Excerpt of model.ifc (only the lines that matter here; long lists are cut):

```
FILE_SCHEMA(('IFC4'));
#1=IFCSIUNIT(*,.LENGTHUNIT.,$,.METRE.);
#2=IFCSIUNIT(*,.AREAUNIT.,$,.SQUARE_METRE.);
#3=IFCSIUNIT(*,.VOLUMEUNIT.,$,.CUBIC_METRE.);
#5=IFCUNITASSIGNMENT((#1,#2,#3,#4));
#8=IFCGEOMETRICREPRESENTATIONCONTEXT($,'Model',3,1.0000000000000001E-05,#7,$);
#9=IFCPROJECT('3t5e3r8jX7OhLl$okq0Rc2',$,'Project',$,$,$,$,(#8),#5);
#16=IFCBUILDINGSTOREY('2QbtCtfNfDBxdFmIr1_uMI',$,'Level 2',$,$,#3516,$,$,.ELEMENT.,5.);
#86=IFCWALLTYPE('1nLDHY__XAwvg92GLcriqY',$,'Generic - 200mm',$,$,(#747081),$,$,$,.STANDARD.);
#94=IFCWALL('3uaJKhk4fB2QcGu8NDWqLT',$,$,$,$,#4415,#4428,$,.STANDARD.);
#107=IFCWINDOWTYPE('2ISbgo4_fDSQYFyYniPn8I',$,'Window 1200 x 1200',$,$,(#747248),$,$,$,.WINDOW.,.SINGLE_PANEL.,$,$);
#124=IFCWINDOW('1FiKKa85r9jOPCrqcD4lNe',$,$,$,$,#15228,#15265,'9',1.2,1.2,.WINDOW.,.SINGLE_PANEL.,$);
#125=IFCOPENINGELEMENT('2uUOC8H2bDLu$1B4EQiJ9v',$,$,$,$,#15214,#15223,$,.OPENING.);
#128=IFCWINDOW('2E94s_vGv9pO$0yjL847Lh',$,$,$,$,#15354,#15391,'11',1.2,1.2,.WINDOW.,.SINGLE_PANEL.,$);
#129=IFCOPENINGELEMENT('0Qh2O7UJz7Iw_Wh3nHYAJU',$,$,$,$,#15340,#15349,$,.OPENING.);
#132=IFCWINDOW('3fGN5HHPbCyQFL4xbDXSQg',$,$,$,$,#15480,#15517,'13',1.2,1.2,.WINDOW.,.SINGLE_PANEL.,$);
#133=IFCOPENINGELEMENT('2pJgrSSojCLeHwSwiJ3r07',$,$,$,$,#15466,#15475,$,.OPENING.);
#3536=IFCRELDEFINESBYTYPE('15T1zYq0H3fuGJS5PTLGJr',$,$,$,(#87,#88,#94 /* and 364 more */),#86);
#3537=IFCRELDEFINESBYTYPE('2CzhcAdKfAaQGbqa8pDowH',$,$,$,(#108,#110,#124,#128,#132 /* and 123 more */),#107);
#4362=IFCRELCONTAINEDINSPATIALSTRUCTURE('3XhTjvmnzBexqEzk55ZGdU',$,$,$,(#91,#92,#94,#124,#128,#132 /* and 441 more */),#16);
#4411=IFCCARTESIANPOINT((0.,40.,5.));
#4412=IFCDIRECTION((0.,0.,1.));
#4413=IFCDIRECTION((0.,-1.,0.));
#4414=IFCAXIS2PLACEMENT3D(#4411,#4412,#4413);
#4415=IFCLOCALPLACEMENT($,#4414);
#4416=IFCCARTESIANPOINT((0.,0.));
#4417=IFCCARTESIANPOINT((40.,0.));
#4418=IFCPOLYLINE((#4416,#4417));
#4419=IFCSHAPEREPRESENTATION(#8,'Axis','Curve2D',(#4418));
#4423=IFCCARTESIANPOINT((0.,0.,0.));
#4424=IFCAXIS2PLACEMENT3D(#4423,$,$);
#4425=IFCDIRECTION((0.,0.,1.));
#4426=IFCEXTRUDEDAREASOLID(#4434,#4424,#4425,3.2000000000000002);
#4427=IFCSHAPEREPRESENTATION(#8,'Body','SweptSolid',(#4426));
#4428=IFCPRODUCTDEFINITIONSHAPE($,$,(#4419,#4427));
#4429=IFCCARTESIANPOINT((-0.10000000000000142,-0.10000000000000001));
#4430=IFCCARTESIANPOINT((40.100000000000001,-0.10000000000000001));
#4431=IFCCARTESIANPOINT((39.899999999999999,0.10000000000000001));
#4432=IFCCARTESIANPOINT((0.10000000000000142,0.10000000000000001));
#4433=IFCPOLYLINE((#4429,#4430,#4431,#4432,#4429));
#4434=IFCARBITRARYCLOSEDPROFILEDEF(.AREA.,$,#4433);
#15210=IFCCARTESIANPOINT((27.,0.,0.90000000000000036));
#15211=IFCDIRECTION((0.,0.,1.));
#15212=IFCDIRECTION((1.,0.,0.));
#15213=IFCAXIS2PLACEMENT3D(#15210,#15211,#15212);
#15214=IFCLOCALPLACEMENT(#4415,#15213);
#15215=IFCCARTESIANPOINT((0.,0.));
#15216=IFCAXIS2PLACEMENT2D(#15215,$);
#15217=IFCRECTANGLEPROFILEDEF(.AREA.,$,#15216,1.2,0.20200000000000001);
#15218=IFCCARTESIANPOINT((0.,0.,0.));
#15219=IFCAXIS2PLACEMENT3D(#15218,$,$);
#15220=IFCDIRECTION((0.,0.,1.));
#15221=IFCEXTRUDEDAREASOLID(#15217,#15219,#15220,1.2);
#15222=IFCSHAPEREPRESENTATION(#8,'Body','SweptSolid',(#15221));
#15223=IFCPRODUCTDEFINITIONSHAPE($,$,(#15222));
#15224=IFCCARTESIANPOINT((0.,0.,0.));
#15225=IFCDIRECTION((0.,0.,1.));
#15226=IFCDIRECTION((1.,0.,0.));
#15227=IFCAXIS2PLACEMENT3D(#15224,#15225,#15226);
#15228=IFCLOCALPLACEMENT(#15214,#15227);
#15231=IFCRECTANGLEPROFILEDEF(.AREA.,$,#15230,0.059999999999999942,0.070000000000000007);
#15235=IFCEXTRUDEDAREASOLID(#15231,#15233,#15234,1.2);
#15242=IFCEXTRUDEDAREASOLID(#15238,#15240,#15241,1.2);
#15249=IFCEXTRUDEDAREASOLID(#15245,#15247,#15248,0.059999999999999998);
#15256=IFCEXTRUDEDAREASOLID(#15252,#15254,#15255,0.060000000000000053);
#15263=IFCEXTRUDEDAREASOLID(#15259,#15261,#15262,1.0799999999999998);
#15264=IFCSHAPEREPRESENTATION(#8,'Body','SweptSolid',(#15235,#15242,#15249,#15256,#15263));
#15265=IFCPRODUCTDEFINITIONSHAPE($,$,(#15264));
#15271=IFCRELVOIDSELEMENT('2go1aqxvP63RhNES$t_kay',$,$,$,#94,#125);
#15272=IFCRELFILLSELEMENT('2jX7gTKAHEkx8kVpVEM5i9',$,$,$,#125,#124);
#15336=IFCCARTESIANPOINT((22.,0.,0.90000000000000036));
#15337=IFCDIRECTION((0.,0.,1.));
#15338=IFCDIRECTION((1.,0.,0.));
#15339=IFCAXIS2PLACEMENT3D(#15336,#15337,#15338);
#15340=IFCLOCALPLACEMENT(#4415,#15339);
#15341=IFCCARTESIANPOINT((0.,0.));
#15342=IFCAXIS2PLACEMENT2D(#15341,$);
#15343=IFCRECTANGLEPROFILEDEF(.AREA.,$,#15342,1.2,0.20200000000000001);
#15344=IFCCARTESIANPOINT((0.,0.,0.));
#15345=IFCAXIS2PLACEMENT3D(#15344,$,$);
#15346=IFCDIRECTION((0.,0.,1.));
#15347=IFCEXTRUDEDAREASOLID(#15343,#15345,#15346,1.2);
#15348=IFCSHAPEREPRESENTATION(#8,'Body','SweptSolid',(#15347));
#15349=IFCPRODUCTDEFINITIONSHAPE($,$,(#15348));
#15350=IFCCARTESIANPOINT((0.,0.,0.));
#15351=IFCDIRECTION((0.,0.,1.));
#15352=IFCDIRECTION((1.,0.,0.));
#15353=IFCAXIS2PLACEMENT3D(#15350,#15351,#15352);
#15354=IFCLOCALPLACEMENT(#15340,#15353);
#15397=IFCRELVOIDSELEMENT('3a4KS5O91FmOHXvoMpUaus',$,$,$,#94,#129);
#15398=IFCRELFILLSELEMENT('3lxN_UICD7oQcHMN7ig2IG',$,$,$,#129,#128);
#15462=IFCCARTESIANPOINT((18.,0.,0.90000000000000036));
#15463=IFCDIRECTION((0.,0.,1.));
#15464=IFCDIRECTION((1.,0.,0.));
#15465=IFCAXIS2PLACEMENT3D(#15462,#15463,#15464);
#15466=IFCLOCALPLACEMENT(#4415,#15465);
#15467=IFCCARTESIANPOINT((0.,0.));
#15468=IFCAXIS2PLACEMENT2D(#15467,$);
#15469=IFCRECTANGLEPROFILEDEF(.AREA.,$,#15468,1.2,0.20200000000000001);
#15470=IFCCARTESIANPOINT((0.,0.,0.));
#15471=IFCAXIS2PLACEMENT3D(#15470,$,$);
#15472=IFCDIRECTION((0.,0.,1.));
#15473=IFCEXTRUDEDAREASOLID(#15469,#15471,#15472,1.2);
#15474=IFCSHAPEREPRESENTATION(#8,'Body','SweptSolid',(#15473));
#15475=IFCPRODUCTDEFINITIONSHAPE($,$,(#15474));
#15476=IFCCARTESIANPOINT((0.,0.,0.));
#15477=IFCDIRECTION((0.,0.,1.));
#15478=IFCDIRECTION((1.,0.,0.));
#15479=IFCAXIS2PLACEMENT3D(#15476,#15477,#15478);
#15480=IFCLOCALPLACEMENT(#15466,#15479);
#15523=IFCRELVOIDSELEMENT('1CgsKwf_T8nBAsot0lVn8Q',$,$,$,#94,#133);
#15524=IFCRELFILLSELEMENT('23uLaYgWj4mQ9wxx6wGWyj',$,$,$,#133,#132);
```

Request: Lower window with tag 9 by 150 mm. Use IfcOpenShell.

```python
import numpy as np
import ifcopenshell
import ifcopenshell.api.geometry
import ifcopenshell.util.placement
import ifcopenshell.util.unit

model = ifcopenshell.open("model.ifc")
unit_scale = ifcopenshell.util.unit.calculate_unit_scale(model)

window = model.by_guid("1FiKKa85r9jOPCrqcD4lNe")
opening = window.FillsVoids[0].RelatingOpeningElement
dz = -0.15 / unit_scale

shift = np.array([0.0, 0.0, dz])
# The window is placed relative to its opening, so it follows when the opening moves.
matrix = ifcopenshell.util.placement.get_local_placement(opening.ObjectPlacement)
matrix[:3, 3] += shift
ifcopenshell.api.geometry.edit_object_placement(
    model, product=opening, matrix=matrix, is_si=False, should_transform_children=True
)

print(f"moved by {dz * unit_scale:+.3f} m")

model.write("model_rev.ifc")
```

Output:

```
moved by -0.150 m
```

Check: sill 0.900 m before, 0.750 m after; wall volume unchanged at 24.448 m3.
